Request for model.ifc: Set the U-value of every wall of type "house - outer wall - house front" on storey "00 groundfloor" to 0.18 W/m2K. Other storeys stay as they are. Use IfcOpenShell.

First a look at what the model holds.

```python
import ifcopenshell
import ifcopenshell.util.element

model = ifcopenshell.open("model.ifc")
print(model.schema)
storey = next(s for s in model.by_type("IfcBuildingStorey") if s.Name == "00 groundfloor")
walls = [e for e in ifcopenshell.util.element.get_decomposition(storey) if e.is_a("IfcWall")]
seen = {}
for e in walls:
    element_type = ifcopenshell.util.element.get_type(e)
    key = (element_type.Name if element_type != e and element_type else None, ifcopenshell.util.element.get_pset(e, "Pset_WallCommon", "ThermalTransmittance"))
    seen[key] = seen.get(key, 0) + 1
for (name, value), count in sorted(seen.items(), key=str):
    print(count, "x", name, "|", value)
```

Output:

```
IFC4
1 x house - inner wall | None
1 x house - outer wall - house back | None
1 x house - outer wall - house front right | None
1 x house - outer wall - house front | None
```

```python
import ifcopenshell
import ifcopenshell.api.pset
import ifcopenshell.util.element

model = ifcopenshell.open("model.ifc")

storey = next(s for s in model.by_type("IfcBuildingStorey") if s.Name == "00 groundfloor")
walls = [e for e in ifcopenshell.util.element.get_decomposition(storey) if e.is_a("IfcWall")]

count = 0
for e in walls:
    element_type = ifcopenshell.util.element.get_type(e)
    if element_type in (None, e) or element_type.Name != "house - outer wall - house front":
        continue
    # add_pset returns the element's existing set when there is one.
    pset = ifcopenshell.api.pset.add_pset(model, product=e, name="Pset_WallCommon")
    ifcopenshell.api.pset.edit_pset(model, pset=pset, properties={"ThermalTransmittance": 0.18})
    count += 1

print(count, "walls updated")

model.write("model_rev.ifc")
```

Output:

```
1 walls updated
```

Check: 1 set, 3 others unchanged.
